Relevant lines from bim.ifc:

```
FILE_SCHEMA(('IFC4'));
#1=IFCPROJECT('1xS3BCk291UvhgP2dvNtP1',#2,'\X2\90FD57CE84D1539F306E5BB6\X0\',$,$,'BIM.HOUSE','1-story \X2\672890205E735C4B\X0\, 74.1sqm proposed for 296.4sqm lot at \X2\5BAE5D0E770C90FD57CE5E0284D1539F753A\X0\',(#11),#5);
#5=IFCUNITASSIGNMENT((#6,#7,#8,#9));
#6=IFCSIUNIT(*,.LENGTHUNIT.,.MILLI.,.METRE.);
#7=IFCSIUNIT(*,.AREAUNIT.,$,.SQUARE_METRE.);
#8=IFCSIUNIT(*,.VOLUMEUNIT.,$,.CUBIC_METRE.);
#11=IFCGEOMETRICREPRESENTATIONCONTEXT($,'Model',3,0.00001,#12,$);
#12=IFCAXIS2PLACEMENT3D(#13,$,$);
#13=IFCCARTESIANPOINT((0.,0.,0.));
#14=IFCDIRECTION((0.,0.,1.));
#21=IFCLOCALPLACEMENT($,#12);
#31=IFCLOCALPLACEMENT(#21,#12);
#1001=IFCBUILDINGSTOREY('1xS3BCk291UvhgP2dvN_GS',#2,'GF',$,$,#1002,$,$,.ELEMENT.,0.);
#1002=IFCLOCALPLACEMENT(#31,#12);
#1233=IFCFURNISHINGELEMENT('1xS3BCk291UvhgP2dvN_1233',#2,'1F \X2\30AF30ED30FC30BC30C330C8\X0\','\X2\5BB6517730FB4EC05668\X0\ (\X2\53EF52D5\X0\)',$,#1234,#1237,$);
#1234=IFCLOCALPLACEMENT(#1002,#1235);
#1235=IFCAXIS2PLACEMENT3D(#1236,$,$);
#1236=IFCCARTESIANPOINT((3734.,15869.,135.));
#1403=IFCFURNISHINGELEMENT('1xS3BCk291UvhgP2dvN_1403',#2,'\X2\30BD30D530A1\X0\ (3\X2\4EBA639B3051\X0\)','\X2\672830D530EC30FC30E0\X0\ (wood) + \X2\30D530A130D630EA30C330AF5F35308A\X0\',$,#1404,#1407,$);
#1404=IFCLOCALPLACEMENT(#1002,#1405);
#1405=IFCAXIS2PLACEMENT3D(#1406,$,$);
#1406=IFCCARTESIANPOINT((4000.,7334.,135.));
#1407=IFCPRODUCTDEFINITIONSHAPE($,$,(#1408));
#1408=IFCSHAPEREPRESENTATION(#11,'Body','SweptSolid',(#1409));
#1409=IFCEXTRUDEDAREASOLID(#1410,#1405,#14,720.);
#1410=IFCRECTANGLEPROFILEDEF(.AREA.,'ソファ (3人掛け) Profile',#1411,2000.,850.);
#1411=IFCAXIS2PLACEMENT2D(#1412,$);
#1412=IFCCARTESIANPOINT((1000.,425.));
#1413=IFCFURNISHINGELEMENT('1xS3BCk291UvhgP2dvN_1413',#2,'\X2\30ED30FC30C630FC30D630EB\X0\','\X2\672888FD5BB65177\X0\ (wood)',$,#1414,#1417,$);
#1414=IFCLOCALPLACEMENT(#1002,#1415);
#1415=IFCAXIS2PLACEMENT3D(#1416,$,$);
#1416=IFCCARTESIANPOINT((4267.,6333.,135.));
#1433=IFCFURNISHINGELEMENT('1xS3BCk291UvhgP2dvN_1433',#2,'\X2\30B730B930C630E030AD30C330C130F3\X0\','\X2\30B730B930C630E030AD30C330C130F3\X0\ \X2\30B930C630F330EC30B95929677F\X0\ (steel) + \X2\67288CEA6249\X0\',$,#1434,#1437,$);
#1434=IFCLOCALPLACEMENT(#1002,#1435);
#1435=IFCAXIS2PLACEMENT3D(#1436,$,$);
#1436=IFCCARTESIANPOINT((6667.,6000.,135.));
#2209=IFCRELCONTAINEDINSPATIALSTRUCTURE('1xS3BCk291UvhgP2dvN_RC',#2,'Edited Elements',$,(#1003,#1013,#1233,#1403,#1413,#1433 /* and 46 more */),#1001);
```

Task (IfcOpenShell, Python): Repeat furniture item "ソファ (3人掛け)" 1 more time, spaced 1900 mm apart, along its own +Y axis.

```python
import ifcopenshell
import ifcopenshell.api.geometry
import ifcopenshell.api.root
import ifcopenshell.util.element
import ifcopenshell.util.placement

model = ifcopenshell.open("bim.ifc")


def reuse_history(source, copy):
    """copy_class also copies each property set's owner history, people and application; keep the originals."""
    for rel in copy.IsDefinedBy:
        if rel.is_a("IfcRelDefinesByProperties") and (history := rel.RelatingPropertyDefinition.OwnerHistory):
            rel.RelatingPropertyDefinition.OwnerHistory = source.OwnerHistory
            ifcopenshell.util.element.remove_deep2(model, history)


source = model.by_guid("1xS3BCk291UvhgP2dvN_1403")
base = ifcopenshell.util.placement.get_local_placement(source.ObjectPlacement)
step = base[:3, 1] * 1900.0

for i in range(1, 2):
    copy = ifcopenshell.api.root.copy_class(model, product=source)
    copy.Representation = ifcopenshell.util.element.copy_deep(
        model, source.Representation, exclude=["IfcGeometricRepresentationContext", "IfcRepresentationMap"]
    )
    reuse_history(source, copy)
    matrix = base.copy()
    matrix[:3, 3] += i * step
    print("added at", matrix[:3, 3].round(3) + 0.0)
    ifcopenshell.api.geometry.edit_object_placement(model, product=copy, matrix=matrix, is_si=False)

model.write("bim-out.ifc")
```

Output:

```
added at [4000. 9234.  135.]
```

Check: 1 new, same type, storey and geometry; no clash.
